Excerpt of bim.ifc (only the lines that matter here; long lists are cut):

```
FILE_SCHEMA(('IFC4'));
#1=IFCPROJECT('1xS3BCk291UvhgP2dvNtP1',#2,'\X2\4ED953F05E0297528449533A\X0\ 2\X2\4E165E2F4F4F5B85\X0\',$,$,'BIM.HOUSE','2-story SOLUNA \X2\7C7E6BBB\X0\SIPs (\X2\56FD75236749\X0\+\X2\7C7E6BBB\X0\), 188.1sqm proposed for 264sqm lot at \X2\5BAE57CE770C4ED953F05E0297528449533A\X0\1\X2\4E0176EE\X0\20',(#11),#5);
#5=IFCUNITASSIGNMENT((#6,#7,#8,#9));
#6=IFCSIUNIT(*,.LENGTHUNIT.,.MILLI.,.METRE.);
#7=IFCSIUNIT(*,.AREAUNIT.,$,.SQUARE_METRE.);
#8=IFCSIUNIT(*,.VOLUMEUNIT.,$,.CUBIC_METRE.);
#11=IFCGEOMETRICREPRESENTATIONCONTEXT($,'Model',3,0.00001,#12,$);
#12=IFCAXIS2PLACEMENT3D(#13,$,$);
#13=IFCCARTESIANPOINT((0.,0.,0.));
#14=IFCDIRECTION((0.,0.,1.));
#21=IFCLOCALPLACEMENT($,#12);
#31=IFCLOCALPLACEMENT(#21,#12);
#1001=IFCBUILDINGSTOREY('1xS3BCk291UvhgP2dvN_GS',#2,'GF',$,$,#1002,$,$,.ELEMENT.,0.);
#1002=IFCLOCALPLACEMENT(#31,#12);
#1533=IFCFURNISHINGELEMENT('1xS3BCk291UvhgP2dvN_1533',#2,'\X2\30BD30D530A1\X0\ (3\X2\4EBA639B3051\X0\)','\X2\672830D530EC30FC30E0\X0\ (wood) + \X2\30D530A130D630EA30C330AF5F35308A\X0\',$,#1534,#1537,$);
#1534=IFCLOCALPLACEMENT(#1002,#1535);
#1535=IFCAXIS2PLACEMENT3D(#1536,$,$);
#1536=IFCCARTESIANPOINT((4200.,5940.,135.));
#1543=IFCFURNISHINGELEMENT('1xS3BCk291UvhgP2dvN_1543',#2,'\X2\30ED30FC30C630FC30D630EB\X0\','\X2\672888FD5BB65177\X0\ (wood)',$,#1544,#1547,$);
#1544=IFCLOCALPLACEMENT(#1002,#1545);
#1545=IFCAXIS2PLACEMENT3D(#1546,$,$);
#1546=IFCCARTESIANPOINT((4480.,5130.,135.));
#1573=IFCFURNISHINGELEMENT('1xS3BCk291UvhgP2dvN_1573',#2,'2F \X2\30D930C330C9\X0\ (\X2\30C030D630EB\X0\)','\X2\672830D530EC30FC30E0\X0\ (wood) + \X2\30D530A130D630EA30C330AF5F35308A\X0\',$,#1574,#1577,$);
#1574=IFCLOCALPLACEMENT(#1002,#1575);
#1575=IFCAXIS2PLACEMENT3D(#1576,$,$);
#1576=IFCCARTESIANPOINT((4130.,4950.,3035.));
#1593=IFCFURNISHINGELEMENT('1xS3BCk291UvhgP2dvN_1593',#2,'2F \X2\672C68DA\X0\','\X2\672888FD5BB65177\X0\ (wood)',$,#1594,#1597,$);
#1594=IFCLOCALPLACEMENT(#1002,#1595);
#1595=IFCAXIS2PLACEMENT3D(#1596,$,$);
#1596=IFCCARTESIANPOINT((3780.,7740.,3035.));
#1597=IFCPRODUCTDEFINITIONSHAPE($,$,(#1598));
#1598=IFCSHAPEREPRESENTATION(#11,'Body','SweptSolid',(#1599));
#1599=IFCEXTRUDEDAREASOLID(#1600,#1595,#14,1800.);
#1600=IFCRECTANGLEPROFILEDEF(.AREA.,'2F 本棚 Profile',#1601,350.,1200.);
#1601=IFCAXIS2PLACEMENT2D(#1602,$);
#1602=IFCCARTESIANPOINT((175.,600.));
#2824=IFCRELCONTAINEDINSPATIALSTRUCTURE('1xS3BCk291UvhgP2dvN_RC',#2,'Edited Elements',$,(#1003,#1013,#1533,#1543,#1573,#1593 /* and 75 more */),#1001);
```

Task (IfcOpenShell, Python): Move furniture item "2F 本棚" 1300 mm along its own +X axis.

```python
import ifcopenshell
import ifcopenshell.api.geometry
import ifcopenshell.util.placement
import ifcopenshell.util.unit

model = ifcopenshell.open("bim.ifc")
unit_scale = ifcopenshell.util.unit.calculate_unit_scale(model)

item = model.by_guid("1xS3BCk291UvhgP2dvN_1593")
matrix = ifcopenshell.util.placement.get_local_placement(item.ObjectPlacement)
matrix[:3, 3] += matrix[:3, 0] * 1.3 / unit_scale
ifcopenshell.api.geometry.edit_object_placement(model, product=item, matrix=matrix, is_si=False)

print(ifcopenshell.util.placement.get_local_placement(item.ObjectPlacement).round(3) + 0.0)

model.write("bim_v2.ifc")
```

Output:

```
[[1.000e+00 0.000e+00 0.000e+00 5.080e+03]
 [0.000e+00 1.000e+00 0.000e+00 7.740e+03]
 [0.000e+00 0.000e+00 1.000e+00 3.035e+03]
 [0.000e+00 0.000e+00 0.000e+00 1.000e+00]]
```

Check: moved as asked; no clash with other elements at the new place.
